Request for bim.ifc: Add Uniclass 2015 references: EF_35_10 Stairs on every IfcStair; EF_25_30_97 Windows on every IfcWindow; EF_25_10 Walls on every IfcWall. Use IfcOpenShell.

First a look at what the model holds.

```python
import ifcopenshell

model = ifcopenshell.open("bim.ifc")
print(model.schema)
print("classifications:", [c.Name for c in model.by_type("IfcClassification")])
for ifc_class in ("IfcDoor", "IfcRoof", "IfcStair", "IfcWall", "IfcWindow"):
    print(ifc_class, len(model.by_type(ifc_class)))
```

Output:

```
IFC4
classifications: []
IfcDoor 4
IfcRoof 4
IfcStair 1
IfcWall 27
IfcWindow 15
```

```python
import ifcopenshell
import ifcopenshell.api.classification

model = ifcopenshell.open("bim.ifc")

system = ifcopenshell.api.classification.add_classification(model, classification="Uniclass 2015")

codes = {
    "IfcStair": ("EF_35_10", "Stairs"),
    "IfcWindow": ("EF_25_30_97", "Windows"),
    "IfcWall": ("EF_25_10", "Walls"),
}
for ifc_class, (code, name) in codes.items():
    products = model.by_type(ifc_class)
    ifcopenshell.api.classification.add_reference(
        model, products=products, classification=system, identification=code, name=name
    )
    print(code, len(products))

model.write("bim_edited.ifc")
```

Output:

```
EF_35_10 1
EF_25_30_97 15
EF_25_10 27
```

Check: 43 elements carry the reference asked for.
